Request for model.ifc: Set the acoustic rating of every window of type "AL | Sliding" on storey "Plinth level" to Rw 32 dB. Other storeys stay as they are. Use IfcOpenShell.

First a look at what the model holds.

```python
import ifcopenshell
import ifcopenshell.util.element

model = ifcopenshell.open("model.ifc")
print(model.schema)
storey = next(s for s in model.by_type("IfcBuildingStorey") if s.Name == "Plinth level")
windows = [e for e in ifcopenshell.util.element.get_decomposition(storey) if e.is_a("IfcWindow")]
seen = {}
for e in windows:
    element_type = ifcopenshell.util.element.get_type(e)
    key = (element_type.Name if element_type != e and element_type else None, ifcopenshell.util.element.get_pset(e, "Pset_WindowCommon", "AcousticRating"))
    seen[key] = seen.get(key, 0) + 1
for (name, value), count in sorted(seen.items(), key=str):
    print(count, "x", name, "|", value)
```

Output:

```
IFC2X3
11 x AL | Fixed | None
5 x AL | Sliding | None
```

```python
import ifcopenshell
import ifcopenshell.api.pset
import ifcopenshell.util.element

model = ifcopenshell.open("model.ifc")

storey = next(s for s in model.by_type("IfcBuildingStorey") if s.Name == "Plinth level")
windows = [e for e in ifcopenshell.util.element.get_decomposition(storey) if e.is_a("IfcWindow")]

count = 0
for e in windows:
    element_type = ifcopenshell.util.element.get_type(e)
    if element_type in (None, e) or element_type.Name != "AL | Sliding":
        continue
    # add_pset returns the element's existing set when there is one.
    pset = ifcopenshell.api.pset.add_pset(model, product=e, name="Pset_WindowCommon")
    ifcopenshell.api.pset.edit_pset(model, pset=pset, properties={"AcousticRating": "Rw 32 dB"})
    count += 1

print(count, "windows updated")

model.write("model_rev.ifc")
```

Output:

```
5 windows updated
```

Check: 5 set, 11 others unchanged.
